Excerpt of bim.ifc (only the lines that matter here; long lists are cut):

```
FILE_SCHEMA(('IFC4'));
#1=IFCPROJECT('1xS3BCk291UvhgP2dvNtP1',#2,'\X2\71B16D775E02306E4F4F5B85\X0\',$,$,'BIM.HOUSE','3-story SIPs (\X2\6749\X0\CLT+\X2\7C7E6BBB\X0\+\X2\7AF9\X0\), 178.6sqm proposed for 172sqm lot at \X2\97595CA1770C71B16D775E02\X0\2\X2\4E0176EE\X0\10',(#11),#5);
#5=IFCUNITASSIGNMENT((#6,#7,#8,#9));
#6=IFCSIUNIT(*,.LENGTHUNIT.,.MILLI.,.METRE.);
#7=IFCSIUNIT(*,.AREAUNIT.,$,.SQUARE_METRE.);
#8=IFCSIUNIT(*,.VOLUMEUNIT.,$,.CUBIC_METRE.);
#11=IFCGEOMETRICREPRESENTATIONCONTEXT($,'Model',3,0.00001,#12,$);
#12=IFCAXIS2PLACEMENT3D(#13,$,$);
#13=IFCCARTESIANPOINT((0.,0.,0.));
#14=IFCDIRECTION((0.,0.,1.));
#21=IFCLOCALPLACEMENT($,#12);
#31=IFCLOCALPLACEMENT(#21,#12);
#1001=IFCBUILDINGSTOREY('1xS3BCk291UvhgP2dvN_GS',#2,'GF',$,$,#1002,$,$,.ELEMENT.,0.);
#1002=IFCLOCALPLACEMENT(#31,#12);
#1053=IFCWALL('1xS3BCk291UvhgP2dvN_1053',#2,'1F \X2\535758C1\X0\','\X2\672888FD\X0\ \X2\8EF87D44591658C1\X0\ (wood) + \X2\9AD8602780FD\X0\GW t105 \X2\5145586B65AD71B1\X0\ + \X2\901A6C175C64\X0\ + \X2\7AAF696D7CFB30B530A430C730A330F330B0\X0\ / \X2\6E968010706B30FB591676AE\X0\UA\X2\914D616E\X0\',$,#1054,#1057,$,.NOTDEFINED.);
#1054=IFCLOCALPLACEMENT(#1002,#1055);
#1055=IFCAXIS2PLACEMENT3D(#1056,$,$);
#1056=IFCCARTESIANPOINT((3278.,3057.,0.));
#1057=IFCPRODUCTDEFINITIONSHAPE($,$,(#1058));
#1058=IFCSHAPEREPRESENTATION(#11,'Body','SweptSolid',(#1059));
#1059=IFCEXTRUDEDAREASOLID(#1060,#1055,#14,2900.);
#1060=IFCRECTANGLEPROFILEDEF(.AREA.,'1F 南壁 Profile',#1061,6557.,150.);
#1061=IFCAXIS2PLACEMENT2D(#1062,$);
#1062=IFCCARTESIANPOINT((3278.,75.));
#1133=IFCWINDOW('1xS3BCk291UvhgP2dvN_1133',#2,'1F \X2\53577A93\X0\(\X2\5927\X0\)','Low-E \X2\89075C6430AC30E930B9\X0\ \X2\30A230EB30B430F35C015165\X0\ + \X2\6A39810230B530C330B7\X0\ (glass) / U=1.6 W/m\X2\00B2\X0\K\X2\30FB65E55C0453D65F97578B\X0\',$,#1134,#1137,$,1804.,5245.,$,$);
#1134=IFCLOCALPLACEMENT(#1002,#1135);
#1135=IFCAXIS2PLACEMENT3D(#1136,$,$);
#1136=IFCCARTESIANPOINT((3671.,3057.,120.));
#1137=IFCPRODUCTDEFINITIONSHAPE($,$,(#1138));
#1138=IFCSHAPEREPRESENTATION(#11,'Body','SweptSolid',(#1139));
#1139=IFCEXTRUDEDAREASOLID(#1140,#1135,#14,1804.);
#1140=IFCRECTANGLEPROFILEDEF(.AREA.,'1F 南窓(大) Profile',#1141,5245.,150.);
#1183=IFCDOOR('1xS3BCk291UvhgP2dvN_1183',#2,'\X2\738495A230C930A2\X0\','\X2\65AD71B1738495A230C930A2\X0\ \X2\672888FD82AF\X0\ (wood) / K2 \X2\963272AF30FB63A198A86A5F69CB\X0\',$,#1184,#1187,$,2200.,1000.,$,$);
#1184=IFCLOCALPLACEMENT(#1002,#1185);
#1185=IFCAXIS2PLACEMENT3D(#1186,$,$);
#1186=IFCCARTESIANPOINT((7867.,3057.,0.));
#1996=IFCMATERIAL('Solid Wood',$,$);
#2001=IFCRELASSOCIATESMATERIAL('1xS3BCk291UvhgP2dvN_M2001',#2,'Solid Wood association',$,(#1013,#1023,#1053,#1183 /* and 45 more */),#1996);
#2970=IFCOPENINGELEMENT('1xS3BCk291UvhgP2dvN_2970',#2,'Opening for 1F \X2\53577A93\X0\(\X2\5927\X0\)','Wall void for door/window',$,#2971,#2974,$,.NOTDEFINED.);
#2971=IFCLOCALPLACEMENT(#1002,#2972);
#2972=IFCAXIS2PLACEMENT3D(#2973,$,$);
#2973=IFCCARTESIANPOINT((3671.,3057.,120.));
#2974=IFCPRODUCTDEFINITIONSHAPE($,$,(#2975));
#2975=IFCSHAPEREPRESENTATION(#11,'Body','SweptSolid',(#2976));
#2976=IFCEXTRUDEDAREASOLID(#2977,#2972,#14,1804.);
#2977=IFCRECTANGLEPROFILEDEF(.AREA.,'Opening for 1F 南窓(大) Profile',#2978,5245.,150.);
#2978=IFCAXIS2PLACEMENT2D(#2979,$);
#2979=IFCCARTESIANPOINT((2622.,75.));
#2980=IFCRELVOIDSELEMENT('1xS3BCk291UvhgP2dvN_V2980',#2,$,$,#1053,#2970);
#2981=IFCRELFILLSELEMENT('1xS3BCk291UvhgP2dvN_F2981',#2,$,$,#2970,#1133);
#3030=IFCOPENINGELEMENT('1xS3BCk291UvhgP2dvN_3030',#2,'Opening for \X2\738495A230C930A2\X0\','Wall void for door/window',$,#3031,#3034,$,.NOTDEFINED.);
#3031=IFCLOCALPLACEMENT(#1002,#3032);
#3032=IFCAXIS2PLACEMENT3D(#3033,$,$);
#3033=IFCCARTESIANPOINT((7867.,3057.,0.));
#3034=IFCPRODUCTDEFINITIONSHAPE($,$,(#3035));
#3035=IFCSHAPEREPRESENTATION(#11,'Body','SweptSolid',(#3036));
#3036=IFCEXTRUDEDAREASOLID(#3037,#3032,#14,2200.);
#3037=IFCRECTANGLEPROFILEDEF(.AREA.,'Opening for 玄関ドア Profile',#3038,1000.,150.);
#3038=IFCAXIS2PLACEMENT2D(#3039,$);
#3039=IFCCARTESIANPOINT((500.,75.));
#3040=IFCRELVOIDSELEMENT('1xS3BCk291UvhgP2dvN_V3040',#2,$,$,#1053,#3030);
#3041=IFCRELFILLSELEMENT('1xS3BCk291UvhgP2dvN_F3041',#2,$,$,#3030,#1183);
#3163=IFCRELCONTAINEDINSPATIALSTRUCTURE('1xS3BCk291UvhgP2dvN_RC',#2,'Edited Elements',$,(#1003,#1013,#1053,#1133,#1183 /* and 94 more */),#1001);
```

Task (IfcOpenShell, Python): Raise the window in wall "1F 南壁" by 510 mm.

```python
import numpy as np
import ifcopenshell
import ifcopenshell.api.geometry
import ifcopenshell.util.placement
import ifcopenshell.util.unit

model = ifcopenshell.open("bim.ifc")
unit_scale = ifcopenshell.util.unit.calculate_unit_scale(model)

window = model.by_guid("1xS3BCk291UvhgP2dvN_1133")
opening = window.FillsVoids[0].RelatingOpeningElement
dz = 510.0

shift = np.array([0.0, 0.0, dz])
# The window is not placed relative to its opening, so move both.
for product in (opening, window):
    matrix = ifcopenshell.util.placement.get_local_placement(product.ObjectPlacement)
    matrix[:3, 3] += shift
    ifcopenshell.api.geometry.edit_object_placement(model, product=product, matrix=matrix, is_si=False)

print(f"moved by {dz * unit_scale:+.3f} m")

model.write("bim_updated.ifc")
```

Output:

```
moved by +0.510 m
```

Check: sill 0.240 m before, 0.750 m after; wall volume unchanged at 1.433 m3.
